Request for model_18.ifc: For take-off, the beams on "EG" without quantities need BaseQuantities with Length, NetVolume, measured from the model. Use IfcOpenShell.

First a look at what the model holds.

```python
import ifcopenshell
import ifcopenshell.util.element
import ifcopenshell.util.unit

model = ifcopenshell.open("model_18.ifc")
print(model.schema)
for unit_type in ("LENGTHUNIT", "AREAUNIT", "VOLUMEUNIT"):
    print(unit_type, ifcopenshell.util.unit.calculate_unit_scale(model, unit_type))
storey = next(s for s in model.by_type("IfcBuildingStorey") if s.Name == "EG")
beams = [e for e in ifcopenshell.util.element.get_decomposition(storey) if e.is_a("IfcBeam")]
for e in sorted(beams, key=lambda e: e.id()):
    print(e.id(), e.is_a(), e.Name, list(ifcopenshell.util.element.get_psets(e, qtos_only=True)), sep=" | ")
```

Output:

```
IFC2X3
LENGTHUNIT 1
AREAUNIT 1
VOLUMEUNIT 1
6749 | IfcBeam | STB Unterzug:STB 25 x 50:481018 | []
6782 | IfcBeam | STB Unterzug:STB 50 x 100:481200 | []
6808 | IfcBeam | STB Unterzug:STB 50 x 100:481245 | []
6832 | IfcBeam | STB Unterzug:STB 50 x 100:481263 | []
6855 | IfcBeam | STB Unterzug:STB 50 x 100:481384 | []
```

```python
import ifcopenshell
import ifcopenshell.api.pset
import ifcopenshell.geom
import ifcopenshell.util.element
import ifcopenshell.util.shape
import ifcopenshell.util.unit

model = ifcopenshell.open("model_18.ifc")
unit_scale = ifcopenshell.util.unit.calculate_unit_scale(model)
volume_scale = ifcopenshell.util.unit.calculate_unit_scale(model, "VOLUMEUNIT")
settings = ifcopenshell.geom.settings()

storey = next(s for s in model.by_type("IfcBuildingStorey") if s.Name == "EG")
beams = [e for e in ifcopenshell.util.element.get_decomposition(storey) if e.is_a("IfcBeam")]

for e in sorted(beams, key=lambda e: e.id()):
    if ifcopenshell.util.element.get_psets(e, qtos_only=True, should_inherit=False):
        continue
    # Geometry comes back in metres, in the element's own axes.
    shape = ifcopenshell.geom.create_shape(settings, e)
    values = {
        "Length": ifcopenshell.util.shape.get_max_xyz(shape.geometry) / unit_scale,
        "NetVolume": ifcopenshell.util.shape.get_volume(shape.geometry) / volume_scale,
    }
    qto = ifcopenshell.api.pset.add_qto(model, product=e, name="BaseQuantities")
    ifcopenshell.api.pset.edit_qto(model, qto=qto, properties=values)
    print(e.id(), {k: round(v, 3) for k, v in values.items()})

model.write("model_18-out.ifc")
```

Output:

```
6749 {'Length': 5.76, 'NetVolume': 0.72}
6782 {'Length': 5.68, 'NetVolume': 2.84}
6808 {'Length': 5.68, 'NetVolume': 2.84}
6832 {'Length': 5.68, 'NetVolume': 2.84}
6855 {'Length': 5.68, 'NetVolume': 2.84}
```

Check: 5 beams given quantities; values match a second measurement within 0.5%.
